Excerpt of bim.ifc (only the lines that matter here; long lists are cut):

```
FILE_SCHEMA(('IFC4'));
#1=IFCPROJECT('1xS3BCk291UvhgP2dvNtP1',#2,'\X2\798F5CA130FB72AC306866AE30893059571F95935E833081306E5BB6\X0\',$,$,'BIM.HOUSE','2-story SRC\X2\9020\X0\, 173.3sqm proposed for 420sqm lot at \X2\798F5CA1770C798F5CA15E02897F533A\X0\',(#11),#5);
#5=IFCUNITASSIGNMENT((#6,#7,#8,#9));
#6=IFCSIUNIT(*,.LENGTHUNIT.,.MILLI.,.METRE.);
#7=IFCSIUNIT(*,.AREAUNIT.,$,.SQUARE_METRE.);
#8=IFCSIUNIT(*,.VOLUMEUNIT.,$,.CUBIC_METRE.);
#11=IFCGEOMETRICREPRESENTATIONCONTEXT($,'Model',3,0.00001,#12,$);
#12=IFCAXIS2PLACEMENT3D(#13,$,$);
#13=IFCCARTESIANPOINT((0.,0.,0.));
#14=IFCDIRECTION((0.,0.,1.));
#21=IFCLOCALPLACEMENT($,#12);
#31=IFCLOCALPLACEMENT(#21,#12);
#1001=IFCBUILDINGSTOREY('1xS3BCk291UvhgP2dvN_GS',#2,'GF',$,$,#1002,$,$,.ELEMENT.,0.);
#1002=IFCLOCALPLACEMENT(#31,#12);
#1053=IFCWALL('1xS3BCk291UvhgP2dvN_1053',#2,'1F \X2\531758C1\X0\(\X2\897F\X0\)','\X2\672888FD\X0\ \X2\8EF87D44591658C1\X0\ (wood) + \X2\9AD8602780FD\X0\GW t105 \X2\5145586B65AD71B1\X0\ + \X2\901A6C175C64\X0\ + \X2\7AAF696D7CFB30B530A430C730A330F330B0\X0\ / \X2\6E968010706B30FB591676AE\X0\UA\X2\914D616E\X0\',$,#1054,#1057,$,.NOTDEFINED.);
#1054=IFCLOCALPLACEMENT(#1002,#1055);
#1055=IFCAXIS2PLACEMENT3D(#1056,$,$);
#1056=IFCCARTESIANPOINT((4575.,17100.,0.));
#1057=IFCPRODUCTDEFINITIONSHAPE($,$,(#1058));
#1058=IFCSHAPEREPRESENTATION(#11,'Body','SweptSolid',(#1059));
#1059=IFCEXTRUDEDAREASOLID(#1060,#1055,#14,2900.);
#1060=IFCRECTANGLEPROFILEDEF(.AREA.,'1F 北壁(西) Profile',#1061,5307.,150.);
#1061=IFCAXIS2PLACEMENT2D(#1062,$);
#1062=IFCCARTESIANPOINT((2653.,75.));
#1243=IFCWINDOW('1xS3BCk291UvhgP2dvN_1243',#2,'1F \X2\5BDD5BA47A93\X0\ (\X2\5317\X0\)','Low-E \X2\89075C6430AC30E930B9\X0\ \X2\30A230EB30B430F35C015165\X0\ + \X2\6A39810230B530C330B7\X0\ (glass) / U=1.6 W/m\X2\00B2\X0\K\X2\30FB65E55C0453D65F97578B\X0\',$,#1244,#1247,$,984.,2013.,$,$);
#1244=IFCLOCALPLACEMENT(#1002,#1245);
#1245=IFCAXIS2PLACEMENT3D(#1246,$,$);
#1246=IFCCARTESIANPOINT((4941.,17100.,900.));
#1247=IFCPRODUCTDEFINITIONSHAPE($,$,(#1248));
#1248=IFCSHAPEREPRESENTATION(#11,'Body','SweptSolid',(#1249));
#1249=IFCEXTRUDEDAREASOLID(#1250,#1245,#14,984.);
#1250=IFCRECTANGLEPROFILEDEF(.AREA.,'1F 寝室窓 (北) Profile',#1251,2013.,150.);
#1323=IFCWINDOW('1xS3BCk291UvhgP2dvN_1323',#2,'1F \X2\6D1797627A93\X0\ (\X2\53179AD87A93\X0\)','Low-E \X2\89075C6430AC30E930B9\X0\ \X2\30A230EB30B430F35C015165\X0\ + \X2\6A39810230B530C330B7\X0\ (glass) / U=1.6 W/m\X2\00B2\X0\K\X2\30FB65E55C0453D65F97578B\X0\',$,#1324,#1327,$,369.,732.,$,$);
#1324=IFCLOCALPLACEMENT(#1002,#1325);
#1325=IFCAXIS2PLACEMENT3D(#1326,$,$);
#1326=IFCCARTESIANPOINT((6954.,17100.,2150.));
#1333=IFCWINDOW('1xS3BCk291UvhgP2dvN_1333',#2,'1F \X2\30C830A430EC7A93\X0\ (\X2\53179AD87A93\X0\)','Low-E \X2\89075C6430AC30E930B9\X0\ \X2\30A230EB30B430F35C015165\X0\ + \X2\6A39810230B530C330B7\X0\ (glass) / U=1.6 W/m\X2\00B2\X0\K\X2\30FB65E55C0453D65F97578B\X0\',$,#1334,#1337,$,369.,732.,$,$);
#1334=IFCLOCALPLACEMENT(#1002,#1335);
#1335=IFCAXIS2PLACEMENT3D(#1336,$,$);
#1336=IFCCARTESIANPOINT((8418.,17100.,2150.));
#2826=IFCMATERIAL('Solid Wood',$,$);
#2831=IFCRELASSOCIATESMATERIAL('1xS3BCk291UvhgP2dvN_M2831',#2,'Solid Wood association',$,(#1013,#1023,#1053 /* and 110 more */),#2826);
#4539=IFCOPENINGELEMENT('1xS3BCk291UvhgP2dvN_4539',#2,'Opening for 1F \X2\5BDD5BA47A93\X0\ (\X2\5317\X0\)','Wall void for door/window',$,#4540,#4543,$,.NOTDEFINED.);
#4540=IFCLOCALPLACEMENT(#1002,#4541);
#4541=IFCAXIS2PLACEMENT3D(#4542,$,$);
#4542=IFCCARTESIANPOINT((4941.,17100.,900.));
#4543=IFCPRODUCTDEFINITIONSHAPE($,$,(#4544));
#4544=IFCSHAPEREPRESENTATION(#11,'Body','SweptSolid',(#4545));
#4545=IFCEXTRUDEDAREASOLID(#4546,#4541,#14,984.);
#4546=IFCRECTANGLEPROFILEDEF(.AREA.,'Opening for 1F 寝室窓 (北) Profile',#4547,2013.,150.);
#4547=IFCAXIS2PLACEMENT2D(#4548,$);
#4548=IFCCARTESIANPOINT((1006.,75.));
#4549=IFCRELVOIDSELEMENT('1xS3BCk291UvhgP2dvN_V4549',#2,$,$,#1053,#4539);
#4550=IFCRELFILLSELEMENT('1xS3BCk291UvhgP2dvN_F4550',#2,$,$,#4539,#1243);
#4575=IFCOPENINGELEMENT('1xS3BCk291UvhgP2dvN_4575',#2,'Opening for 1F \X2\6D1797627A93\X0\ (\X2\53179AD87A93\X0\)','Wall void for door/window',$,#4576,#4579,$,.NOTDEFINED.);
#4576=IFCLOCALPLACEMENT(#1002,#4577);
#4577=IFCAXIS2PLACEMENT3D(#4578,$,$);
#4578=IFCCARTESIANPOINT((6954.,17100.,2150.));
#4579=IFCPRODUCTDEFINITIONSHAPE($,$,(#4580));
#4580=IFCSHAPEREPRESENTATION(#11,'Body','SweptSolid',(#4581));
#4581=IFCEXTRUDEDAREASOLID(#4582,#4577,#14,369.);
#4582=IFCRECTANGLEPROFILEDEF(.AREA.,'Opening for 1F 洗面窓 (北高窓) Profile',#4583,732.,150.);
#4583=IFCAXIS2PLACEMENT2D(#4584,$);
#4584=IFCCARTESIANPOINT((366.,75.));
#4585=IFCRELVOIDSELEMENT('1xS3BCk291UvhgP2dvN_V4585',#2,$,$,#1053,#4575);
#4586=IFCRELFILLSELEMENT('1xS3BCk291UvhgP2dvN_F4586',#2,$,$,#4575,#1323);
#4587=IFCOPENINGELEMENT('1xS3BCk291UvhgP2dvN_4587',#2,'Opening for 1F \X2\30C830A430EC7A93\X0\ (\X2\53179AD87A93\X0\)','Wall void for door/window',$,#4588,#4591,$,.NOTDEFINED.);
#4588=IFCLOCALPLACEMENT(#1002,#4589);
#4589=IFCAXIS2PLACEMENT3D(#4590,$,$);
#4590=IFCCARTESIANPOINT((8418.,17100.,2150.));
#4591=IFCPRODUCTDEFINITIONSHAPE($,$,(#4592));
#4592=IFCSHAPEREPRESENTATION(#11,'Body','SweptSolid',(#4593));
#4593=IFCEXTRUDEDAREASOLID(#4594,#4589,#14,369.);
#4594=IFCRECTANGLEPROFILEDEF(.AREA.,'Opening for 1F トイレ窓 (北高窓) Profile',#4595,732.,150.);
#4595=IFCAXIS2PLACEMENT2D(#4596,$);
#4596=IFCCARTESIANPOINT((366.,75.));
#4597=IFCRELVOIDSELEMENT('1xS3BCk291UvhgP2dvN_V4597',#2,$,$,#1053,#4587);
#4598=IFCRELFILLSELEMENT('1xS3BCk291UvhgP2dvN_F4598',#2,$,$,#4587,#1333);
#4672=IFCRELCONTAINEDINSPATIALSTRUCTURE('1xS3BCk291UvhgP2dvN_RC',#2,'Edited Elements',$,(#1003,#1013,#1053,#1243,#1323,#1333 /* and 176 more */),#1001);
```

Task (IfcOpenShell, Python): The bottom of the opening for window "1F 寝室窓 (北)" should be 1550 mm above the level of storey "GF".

```python
import numpy as np
import ifcopenshell
import ifcopenshell.api.geometry
import ifcopenshell.geom
import ifcopenshell.util.element
import ifcopenshell.util.placement
import ifcopenshell.util.shape
import ifcopenshell.util.unit

model = ifcopenshell.open("bim.ifc")
unit_scale = ifcopenshell.util.unit.calculate_unit_scale(model)

window = model.by_id(1243)
opening = window.FillsVoids[0].RelatingOpeningElement
storey = ifcopenshell.util.element.get_container(window, ifc_class="IfcBuildingStorey")
level = ifcopenshell.util.placement.get_local_placement(storey.ObjectPlacement)[2, 3]

# The opening's origin need not be at the sill, so measure its lowest point.
shape = ifcopenshell.geom.create_shape(ifcopenshell.geom.settings(), opening)
bottom = ifcopenshell.util.shape.get_shape_bottom_elevation(shape, shape.geometry) / unit_scale
dz = level + 1.55 / unit_scale - bottom

shift = np.array([0.0, 0.0, dz])
# The window is not placed relative to its opening, so move both.
for product in (opening, window):
    matrix = ifcopenshell.util.placement.get_local_placement(product.ObjectPlacement)
    matrix[:3, 3] += shift
    ifcopenshell.api.geometry.edit_object_placement(model, product=product, matrix=matrix, is_si=False)

print(f"moved by {dz * unit_scale:+.3f} m")

model.write("bim_v2.ifc")
```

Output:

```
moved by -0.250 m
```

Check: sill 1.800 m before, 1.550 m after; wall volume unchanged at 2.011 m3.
